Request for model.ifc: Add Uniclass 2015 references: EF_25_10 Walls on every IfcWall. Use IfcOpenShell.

First a look at what the model holds.

```python
import ifcopenshell

model = ifcopenshell.open("model.ifc")
print(model.schema)
print("classifications:", [c.Name for c in model.by_type("IfcClassification")])
for ifc_class in ("IfcDoor", "IfcRoof", "IfcStair", "IfcWall", "IfcWindow"):
    print(ifc_class, len(model.by_type(ifc_class)))
```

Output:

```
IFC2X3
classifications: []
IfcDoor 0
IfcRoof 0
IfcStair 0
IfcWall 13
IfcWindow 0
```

```python
import ifcopenshell
import ifcopenshell.api.classification

model = ifcopenshell.open("model.ifc")

# IFC2X3 requires Source and Edition and has no link from the project to the system.
system = model.create_entity("IfcClassification", Source="NBS", Edition="2015", Name="Uniclass 2015")

codes = {
    "IfcWall": ("EF_25_10", "Walls"),
}
for ifc_class, (code, name) in codes.items():
    products = model.by_type(ifc_class)
    ifcopenshell.api.classification.add_reference(
        model, products=products, classification=system, identification=code, name=name
    )
    print(code, len(products))

model.write("model-out.ifc")
```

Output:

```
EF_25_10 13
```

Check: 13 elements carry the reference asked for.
